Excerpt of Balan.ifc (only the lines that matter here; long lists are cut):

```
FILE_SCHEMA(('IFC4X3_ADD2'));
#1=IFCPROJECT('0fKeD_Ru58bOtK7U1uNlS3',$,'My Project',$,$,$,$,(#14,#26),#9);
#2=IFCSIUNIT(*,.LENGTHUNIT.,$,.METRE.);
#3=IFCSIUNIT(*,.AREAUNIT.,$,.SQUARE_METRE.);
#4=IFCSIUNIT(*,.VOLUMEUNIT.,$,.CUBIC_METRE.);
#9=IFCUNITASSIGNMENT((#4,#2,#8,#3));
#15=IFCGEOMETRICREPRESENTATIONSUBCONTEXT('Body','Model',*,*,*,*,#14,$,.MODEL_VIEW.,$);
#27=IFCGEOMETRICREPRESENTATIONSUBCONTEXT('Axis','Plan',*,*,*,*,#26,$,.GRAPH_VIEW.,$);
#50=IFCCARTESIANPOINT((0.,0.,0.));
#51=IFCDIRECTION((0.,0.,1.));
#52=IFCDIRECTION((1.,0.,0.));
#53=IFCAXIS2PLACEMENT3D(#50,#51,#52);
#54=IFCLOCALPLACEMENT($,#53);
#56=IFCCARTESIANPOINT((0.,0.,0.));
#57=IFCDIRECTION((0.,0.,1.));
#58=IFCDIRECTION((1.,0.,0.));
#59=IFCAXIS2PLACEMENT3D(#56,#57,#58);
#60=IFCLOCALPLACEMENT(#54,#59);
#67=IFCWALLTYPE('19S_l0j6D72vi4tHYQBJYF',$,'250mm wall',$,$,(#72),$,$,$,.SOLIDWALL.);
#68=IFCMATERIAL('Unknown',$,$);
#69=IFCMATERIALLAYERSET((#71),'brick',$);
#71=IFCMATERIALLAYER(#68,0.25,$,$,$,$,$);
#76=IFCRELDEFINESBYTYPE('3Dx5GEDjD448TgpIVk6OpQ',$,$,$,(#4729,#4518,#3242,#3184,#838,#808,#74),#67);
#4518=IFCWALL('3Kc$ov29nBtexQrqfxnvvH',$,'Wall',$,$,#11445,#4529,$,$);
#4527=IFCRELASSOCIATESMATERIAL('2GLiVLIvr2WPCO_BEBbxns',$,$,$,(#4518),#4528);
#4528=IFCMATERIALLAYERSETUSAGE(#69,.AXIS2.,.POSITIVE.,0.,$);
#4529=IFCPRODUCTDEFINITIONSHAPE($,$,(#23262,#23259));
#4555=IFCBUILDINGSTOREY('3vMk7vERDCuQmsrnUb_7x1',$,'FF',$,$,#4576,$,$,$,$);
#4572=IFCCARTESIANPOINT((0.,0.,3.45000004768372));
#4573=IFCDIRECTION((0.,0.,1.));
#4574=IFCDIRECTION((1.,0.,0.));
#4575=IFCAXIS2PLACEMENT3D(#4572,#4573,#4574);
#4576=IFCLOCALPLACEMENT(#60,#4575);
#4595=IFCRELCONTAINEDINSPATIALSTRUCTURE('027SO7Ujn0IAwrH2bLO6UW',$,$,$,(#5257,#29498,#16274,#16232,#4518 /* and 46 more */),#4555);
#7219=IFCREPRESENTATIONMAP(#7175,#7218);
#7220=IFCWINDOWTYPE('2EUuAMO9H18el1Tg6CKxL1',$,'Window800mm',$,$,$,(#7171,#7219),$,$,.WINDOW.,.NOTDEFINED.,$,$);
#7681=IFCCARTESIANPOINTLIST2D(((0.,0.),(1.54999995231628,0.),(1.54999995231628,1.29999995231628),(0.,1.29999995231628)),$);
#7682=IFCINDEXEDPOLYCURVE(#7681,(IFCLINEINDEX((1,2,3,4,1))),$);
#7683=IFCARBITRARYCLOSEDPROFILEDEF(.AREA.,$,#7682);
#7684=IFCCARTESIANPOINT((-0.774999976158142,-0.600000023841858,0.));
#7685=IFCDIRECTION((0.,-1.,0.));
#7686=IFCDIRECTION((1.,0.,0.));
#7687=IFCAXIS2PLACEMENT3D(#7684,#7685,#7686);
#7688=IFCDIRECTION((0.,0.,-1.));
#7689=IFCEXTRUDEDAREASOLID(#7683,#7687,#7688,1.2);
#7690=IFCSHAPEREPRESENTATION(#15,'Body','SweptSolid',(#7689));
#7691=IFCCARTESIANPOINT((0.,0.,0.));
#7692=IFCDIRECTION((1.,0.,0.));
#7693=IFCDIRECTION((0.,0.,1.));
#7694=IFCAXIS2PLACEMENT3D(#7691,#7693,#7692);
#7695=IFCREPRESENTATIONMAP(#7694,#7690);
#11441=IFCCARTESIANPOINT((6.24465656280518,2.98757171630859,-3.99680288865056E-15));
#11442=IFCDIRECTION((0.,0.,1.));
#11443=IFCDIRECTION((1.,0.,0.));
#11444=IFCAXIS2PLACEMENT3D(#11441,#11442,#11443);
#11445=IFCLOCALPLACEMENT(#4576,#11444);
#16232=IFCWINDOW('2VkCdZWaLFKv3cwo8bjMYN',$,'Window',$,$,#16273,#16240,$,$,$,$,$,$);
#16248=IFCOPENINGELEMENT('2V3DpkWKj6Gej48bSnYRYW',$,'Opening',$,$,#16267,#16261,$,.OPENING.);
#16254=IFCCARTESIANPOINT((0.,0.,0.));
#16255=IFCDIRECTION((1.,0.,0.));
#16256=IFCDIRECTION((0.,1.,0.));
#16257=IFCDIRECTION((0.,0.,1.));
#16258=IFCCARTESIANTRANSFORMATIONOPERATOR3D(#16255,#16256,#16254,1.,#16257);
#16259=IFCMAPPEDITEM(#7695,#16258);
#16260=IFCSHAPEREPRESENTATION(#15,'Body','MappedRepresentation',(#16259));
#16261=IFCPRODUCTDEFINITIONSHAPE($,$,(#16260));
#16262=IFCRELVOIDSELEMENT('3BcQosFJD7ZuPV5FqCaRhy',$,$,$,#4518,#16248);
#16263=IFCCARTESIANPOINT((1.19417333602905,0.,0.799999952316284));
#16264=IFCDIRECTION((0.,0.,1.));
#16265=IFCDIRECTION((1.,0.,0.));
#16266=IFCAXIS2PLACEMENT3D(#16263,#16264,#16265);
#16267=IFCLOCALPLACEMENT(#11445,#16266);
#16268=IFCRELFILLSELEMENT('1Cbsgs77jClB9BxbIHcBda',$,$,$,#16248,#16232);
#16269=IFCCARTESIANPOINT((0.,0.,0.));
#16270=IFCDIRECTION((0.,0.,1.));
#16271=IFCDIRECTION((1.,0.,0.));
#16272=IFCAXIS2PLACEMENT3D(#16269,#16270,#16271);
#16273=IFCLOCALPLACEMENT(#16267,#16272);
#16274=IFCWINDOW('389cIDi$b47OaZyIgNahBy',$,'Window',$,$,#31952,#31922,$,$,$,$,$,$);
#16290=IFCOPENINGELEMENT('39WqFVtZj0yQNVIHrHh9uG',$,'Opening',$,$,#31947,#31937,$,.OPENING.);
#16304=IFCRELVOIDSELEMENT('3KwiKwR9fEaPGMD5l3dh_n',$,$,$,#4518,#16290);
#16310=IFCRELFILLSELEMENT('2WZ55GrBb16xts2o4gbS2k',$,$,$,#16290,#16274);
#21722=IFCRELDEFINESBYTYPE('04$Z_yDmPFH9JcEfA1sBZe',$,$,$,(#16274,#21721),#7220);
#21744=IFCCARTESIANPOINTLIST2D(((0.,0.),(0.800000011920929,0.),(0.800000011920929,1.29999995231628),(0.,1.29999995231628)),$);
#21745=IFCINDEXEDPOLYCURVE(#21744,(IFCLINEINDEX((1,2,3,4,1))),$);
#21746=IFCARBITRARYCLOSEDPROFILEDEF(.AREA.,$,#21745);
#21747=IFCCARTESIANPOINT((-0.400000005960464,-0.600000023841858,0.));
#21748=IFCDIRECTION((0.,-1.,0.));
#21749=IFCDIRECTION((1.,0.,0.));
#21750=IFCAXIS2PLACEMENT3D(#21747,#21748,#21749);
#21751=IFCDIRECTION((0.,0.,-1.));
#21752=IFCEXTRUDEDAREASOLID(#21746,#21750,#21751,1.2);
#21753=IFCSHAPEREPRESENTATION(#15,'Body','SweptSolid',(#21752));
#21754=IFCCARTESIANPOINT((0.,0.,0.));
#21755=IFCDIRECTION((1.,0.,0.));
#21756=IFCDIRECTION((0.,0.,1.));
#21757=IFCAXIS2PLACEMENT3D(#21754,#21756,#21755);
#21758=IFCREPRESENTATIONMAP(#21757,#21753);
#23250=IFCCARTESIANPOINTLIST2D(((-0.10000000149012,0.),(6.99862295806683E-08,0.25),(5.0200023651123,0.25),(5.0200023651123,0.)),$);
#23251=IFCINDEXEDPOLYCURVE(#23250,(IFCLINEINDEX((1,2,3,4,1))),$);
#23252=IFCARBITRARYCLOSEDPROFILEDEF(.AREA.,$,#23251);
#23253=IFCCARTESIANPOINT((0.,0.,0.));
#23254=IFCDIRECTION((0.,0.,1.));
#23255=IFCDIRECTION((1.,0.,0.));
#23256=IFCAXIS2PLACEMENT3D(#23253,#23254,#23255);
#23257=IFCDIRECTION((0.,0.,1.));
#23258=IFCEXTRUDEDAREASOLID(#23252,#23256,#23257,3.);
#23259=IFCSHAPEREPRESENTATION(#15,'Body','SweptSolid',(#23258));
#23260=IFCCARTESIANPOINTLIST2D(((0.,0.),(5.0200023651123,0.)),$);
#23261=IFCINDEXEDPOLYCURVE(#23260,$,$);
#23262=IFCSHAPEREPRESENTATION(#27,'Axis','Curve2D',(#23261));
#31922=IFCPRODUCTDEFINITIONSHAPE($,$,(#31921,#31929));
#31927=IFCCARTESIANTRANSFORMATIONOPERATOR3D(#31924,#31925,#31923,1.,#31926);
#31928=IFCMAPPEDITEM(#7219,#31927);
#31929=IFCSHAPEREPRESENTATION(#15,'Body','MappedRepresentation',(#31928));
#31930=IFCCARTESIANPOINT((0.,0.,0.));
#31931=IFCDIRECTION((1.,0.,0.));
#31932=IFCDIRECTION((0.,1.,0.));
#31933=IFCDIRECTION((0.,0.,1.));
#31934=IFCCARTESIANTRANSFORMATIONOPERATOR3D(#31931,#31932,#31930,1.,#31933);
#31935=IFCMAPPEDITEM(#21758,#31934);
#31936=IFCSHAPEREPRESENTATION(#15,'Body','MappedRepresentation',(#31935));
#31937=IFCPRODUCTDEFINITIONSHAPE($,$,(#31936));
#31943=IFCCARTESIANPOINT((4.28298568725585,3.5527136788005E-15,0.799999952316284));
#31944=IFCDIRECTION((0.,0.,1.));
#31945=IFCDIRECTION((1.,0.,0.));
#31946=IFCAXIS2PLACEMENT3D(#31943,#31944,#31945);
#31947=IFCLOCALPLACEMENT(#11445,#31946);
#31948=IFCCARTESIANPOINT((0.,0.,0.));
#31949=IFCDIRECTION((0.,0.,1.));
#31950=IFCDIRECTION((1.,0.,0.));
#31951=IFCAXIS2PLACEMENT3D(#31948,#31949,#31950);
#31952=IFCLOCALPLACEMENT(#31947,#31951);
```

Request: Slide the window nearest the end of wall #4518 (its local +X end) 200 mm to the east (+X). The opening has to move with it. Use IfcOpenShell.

```python
import ifcopenshell
import ifcopenshell.api.geometry
import ifcopenshell.util.placement
import ifcopenshell.util.unit

model = ifcopenshell.open("Balan.ifc")
unit_scale = ifcopenshell.util.unit.calculate_unit_scale(model)

window = model.by_guid("389cIDi$b47OaZyIgNahBy")
opening = window.FillsVoids[0].RelatingOpeningElement
wall = opening.VoidsElements[0].RelatingBuildingElement

wall_matrix = ifcopenshell.util.placement.get_local_placement(wall.ObjectPlacement)
shift = wall_matrix[:3, 0] * 0.2 / unit_scale
before = ifcopenshell.util.placement.get_local_placement(window.ObjectPlacement)[:3, 3].copy()

# The window is placed relative to its opening, so it follows when the opening moves.
matrix = ifcopenshell.util.placement.get_local_placement(opening.ObjectPlacement)
matrix[:3, 3] += shift
ifcopenshell.api.geometry.edit_object_placement(
    model, product=opening, matrix=matrix, is_si=False, should_transform_children=True
)

after = ifcopenshell.util.placement.get_local_placement(window.ObjectPlacement)[:3, 3]
print("window moved by", (after - before).round(3) + 0.0)

model.write("Balan_edited.ifc")
```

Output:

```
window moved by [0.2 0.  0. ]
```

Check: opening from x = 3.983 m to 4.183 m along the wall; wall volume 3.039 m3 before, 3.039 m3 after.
